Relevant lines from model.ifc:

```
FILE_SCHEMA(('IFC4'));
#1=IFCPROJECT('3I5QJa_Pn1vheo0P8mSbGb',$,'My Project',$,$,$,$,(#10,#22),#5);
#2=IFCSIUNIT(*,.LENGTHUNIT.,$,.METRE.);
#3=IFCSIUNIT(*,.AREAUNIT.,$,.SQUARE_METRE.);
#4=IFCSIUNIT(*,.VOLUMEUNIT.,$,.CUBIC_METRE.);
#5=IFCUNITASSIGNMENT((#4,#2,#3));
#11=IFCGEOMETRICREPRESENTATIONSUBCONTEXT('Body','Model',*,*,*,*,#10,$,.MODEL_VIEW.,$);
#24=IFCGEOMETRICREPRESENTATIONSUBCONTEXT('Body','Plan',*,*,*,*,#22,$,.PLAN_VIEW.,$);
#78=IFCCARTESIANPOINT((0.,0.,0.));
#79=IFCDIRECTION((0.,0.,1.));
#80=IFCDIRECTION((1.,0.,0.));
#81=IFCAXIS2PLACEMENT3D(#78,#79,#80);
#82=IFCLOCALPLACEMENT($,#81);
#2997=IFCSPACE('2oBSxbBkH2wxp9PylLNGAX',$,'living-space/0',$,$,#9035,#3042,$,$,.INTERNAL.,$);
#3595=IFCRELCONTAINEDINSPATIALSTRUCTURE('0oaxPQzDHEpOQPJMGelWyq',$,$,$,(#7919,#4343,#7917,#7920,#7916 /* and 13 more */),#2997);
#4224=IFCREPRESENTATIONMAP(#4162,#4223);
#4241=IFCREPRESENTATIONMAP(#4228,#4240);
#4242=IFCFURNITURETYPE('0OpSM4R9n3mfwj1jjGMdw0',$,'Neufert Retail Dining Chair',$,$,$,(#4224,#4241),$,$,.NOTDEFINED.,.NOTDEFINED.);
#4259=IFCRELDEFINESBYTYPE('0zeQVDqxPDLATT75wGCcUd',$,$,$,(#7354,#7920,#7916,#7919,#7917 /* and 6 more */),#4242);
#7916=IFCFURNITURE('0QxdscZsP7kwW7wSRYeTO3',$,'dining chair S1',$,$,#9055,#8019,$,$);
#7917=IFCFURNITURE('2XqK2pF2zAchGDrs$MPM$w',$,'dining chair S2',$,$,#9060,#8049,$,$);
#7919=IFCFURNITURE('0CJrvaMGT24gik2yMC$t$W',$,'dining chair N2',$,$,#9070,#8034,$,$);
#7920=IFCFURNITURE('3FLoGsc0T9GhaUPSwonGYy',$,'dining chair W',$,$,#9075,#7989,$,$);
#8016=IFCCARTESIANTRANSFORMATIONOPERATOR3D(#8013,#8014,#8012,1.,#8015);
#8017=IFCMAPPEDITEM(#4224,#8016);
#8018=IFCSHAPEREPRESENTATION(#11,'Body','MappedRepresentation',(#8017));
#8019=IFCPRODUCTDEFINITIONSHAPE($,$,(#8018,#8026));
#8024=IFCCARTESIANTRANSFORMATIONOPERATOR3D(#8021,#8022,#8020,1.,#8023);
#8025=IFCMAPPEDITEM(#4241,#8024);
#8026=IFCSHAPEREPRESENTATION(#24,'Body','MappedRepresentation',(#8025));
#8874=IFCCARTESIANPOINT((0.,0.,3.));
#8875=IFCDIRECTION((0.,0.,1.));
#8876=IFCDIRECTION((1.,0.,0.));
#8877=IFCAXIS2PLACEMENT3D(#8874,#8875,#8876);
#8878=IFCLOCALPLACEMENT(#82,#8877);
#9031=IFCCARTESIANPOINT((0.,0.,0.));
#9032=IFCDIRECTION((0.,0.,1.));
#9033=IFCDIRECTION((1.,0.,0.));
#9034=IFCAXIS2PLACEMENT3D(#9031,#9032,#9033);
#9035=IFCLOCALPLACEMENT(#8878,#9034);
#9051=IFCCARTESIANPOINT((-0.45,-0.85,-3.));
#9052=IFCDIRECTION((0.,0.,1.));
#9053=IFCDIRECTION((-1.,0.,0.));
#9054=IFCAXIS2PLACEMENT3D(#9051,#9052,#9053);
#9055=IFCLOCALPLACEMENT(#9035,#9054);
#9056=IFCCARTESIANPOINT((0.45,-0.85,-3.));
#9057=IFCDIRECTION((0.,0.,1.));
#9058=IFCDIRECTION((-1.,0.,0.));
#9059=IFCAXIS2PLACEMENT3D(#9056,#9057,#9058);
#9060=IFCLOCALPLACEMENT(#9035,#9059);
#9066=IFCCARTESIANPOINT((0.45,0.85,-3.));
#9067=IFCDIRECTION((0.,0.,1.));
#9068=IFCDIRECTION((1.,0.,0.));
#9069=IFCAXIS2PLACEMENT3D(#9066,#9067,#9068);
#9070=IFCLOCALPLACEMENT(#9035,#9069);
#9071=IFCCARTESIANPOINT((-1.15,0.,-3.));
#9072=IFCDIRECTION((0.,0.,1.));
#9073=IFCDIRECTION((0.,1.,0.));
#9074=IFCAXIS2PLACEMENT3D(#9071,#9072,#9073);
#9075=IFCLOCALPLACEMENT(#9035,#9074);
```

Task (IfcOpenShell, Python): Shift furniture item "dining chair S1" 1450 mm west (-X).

```python
import ifcopenshell
import ifcopenshell.api.geometry
import ifcopenshell.util.placement

model = ifcopenshell.open("model.ifc")

item = model.by_guid("0QxdscZsP7kwW7wSRYeTO3")
matrix = ifcopenshell.util.placement.get_local_placement(item.ObjectPlacement)
matrix[0, 3] -= 1.45
ifcopenshell.api.geometry.edit_object_placement(model, product=item, matrix=matrix, is_si=False)

print(ifcopenshell.util.placement.get_local_placement(item.ObjectPlacement).round(3) + 0.0)

model.write("model-out.ifc")
```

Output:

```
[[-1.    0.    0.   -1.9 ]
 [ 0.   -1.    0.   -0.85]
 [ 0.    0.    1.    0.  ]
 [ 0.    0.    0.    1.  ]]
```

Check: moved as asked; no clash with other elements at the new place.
